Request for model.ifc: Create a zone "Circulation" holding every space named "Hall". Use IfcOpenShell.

First a look at what the model holds.

```python
import ifcopenshell

model = ifcopenshell.open("model.ifc")
print(model.schema)
seen = {}
for space in model.by_type("IfcSpace"):
    seen[space.LongName] = seen.get(space.LongName, 0) + 1
for name, count in sorted(seen.items(), key=str):
    print(count, "x", name)
print("zones:", [z.Name for z in model.by_type("IfcZone")][:20])
```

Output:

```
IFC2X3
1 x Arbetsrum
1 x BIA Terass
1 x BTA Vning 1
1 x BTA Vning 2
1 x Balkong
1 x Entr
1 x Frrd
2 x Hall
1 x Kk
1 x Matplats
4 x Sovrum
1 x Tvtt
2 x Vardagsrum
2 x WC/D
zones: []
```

```python
import ifcopenshell
import ifcopenshell.api.group
import ifcopenshell.api.root

model = ifcopenshell.open("model.ifc")

names = {"Hall"}
spaces = [s for s in model.by_type("IfcSpace") if s.LongName in names]

zone = ifcopenshell.api.root.create_entity(model, ifc_class="IfcZone", name="Circulation")
ifcopenshell.api.group.assign_group(model, products=spaces, group=zone)
print(len(spaces), "spaces in", zone.Name)

model.write("model_edited.ifc")
```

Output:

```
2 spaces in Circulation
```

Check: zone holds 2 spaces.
